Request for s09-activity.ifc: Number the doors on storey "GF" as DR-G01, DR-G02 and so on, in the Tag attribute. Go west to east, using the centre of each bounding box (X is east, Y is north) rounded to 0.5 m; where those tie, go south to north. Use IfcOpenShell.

First a look at what the model holds.

```python
import ifcopenshell
import ifcopenshell.util.element
import ifcopenshell.util.placement

model = ifcopenshell.open("s09-activity.ifc")
print(model.schema)
storey = next(s for s in model.by_type("IfcBuildingStorey") if s.Name == "GF")
doors = [e for e in ifcopenshell.util.element.get_decomposition(storey) if e.is_a("IfcDoor")]
for e in sorted(doors, key=lambda e: e.id()):
    origin = ifcopenshell.util.placement.get_local_placement(e.ObjectPlacement)[:3, 3]
    print(e.id(), e.Tag, e.Name, origin.round(2) + 0.0, sep=" | ")
```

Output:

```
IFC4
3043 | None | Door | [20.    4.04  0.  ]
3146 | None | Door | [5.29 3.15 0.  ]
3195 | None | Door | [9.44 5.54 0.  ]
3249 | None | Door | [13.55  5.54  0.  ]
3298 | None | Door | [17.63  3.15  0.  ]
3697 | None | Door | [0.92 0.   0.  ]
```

```python
import ifcopenshell
import ifcopenshell.geom
import ifcopenshell.util.element
import ifcopenshell.util.shape

model = ifcopenshell.open("s09-activity.ifc")
settings = ifcopenshell.geom.settings()
settings.set("use-world-coords", True)


def centre(element):
    shape = ifcopenshell.geom.create_shape(settings, element)
    return ifcopenshell.util.shape.get_bbox_centroid(shape.geometry)


storey = next(s for s in model.by_type("IfcBuildingStorey") if s.Name == "GF")
doors = [e for e in ifcopenshell.util.element.get_decomposition(storey) if e.is_a("IfcDoor")]

# Insertion points can sit at a corner or the storey origin, so sort by the geometry (in metres).
centres = {e: centre(e) for e in doors}
doors.sort(key=lambda e: (round(centres[e][0] / 0.5), centres[e][1]))

for i, e in enumerate(doors, start=1):
    number = f"DR-G{i:02d}"
    e.Tag = number
    print(e.id(), number)

model.write("s09-activity-out.ifc")
```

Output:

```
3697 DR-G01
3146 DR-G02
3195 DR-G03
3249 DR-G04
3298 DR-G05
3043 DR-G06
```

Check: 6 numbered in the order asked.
